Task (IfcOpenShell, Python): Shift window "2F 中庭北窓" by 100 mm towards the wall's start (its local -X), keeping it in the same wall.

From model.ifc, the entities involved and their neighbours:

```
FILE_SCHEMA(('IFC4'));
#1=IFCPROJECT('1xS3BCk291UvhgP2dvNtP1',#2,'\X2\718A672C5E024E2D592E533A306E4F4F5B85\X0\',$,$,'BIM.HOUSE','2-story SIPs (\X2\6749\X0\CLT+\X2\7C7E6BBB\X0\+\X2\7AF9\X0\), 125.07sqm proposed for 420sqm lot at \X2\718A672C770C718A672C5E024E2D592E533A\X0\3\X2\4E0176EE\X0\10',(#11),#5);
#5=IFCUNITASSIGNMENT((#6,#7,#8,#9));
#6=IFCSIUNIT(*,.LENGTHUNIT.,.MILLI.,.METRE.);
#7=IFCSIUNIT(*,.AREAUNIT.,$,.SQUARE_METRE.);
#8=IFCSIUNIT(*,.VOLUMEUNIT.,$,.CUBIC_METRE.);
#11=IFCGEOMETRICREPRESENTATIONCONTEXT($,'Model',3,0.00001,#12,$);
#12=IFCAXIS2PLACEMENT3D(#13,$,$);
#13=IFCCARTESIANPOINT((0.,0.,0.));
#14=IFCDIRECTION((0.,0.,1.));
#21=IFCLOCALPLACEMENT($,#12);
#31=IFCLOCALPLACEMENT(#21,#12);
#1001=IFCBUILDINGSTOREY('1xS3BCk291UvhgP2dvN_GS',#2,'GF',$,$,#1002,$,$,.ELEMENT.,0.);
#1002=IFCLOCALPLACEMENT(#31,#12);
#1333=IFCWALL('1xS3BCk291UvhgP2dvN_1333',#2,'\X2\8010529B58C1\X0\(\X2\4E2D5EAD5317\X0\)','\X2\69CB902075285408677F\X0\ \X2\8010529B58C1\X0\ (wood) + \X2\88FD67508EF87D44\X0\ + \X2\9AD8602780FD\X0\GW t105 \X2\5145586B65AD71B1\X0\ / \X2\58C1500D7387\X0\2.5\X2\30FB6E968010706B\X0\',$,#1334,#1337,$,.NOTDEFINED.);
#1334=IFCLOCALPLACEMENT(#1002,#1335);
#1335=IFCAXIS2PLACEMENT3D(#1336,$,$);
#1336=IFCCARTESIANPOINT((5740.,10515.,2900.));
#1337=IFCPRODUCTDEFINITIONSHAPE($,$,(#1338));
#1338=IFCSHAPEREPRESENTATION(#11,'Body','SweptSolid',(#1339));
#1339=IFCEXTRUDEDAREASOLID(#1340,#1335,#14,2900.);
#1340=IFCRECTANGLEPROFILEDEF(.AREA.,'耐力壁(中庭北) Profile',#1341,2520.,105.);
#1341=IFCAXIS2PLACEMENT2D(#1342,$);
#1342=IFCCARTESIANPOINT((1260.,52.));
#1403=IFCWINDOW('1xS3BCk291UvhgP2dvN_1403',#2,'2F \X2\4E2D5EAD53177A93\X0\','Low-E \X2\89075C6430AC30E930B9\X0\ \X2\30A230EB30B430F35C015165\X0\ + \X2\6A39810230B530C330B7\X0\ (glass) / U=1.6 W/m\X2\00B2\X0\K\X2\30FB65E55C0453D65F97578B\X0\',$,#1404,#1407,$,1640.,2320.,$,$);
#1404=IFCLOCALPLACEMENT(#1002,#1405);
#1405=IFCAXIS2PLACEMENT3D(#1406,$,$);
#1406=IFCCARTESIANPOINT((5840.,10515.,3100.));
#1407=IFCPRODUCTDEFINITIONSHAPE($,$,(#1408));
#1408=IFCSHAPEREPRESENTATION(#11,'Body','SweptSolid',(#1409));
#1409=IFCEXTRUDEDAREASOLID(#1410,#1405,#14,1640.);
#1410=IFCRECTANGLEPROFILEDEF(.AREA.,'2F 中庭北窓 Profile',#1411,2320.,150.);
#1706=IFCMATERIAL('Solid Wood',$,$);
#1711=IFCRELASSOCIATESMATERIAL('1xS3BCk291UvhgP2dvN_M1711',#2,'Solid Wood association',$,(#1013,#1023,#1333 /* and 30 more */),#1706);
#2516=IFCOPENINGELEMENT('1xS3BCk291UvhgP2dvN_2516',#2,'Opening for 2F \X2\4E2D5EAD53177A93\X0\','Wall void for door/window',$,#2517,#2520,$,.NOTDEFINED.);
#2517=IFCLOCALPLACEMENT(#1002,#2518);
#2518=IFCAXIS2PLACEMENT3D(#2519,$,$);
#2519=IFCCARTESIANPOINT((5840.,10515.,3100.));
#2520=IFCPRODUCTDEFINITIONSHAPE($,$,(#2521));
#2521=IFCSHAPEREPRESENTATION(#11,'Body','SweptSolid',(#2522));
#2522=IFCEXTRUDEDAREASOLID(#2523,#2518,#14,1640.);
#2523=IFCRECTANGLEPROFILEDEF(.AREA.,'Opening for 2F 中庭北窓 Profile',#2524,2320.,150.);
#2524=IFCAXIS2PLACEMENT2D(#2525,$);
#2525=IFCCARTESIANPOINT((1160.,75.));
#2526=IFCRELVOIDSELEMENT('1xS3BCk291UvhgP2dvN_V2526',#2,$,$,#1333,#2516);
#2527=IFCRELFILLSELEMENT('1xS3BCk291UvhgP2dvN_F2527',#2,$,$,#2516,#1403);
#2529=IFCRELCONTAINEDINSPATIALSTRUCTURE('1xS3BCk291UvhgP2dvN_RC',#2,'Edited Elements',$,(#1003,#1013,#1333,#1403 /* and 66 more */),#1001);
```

```python
import ifcopenshell
import ifcopenshell.api.geometry
import ifcopenshell.util.placement
import ifcopenshell.util.unit

model = ifcopenshell.open("model.ifc")
unit_scale = ifcopenshell.util.unit.calculate_unit_scale(model)

window = model.by_id(1403)
opening = window.FillsVoids[0].RelatingOpeningElement
wall = opening.VoidsElements[0].RelatingBuildingElement

wall_matrix = ifcopenshell.util.placement.get_local_placement(wall.ObjectPlacement)
shift = wall_matrix[:3, 0] * -0.1 / unit_scale
before = ifcopenshell.util.placement.get_local_placement(window.ObjectPlacement)[:3, 3].copy()

# The window is not placed relative to its opening, so move both.
for product in (opening, window):
    matrix = ifcopenshell.util.placement.get_local_placement(product.ObjectPlacement)
    matrix[:3, 3] += shift
    ifcopenshell.api.geometry.edit_object_placement(model, product=product, matrix=matrix, is_si=False)

after = ifcopenshell.util.placement.get_local_placement(window.ObjectPlacement)[:3, 3]
print("window moved by", (after - before).round(3) + 0.0)

model.write("model_edited.ifc")
```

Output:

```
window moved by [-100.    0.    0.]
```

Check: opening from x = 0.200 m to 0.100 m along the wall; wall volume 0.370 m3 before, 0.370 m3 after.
